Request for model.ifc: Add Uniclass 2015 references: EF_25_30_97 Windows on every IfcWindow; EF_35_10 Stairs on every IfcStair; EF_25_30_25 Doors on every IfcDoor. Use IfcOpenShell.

First a look at what the model holds.

```python
import ifcopenshell

model = ifcopenshell.open("model.ifc")
print(model.schema)
print("classifications:", [c.Name for c in model.by_type("IfcClassification")])
for ifc_class in ("IfcDoor", "IfcRoof", "IfcStair", "IfcWall", "IfcWindow"):
    print(ifc_class, len(model.by_type(ifc_class)))
```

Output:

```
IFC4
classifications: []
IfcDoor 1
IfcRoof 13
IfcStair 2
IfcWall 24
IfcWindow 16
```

```python
import ifcopenshell
import ifcopenshell.api.classification

model = ifcopenshell.open("model.ifc")

system = ifcopenshell.api.classification.add_classification(model, classification="Uniclass 2015")

codes = {
    "IfcWindow": ("EF_25_30_97", "Windows"),
    "IfcStair": ("EF_35_10", "Stairs"),
    "IfcDoor": ("EF_25_30_25", "Doors"),
}
for ifc_class, (code, name) in codes.items():
    products = model.by_type(ifc_class)
    ifcopenshell.api.classification.add_reference(
        model, products=products, classification=system, identification=code, name=name
    )
    print(code, len(products))

model.write("model_v2.ifc")
```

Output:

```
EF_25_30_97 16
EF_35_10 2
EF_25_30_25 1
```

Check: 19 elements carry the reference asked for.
